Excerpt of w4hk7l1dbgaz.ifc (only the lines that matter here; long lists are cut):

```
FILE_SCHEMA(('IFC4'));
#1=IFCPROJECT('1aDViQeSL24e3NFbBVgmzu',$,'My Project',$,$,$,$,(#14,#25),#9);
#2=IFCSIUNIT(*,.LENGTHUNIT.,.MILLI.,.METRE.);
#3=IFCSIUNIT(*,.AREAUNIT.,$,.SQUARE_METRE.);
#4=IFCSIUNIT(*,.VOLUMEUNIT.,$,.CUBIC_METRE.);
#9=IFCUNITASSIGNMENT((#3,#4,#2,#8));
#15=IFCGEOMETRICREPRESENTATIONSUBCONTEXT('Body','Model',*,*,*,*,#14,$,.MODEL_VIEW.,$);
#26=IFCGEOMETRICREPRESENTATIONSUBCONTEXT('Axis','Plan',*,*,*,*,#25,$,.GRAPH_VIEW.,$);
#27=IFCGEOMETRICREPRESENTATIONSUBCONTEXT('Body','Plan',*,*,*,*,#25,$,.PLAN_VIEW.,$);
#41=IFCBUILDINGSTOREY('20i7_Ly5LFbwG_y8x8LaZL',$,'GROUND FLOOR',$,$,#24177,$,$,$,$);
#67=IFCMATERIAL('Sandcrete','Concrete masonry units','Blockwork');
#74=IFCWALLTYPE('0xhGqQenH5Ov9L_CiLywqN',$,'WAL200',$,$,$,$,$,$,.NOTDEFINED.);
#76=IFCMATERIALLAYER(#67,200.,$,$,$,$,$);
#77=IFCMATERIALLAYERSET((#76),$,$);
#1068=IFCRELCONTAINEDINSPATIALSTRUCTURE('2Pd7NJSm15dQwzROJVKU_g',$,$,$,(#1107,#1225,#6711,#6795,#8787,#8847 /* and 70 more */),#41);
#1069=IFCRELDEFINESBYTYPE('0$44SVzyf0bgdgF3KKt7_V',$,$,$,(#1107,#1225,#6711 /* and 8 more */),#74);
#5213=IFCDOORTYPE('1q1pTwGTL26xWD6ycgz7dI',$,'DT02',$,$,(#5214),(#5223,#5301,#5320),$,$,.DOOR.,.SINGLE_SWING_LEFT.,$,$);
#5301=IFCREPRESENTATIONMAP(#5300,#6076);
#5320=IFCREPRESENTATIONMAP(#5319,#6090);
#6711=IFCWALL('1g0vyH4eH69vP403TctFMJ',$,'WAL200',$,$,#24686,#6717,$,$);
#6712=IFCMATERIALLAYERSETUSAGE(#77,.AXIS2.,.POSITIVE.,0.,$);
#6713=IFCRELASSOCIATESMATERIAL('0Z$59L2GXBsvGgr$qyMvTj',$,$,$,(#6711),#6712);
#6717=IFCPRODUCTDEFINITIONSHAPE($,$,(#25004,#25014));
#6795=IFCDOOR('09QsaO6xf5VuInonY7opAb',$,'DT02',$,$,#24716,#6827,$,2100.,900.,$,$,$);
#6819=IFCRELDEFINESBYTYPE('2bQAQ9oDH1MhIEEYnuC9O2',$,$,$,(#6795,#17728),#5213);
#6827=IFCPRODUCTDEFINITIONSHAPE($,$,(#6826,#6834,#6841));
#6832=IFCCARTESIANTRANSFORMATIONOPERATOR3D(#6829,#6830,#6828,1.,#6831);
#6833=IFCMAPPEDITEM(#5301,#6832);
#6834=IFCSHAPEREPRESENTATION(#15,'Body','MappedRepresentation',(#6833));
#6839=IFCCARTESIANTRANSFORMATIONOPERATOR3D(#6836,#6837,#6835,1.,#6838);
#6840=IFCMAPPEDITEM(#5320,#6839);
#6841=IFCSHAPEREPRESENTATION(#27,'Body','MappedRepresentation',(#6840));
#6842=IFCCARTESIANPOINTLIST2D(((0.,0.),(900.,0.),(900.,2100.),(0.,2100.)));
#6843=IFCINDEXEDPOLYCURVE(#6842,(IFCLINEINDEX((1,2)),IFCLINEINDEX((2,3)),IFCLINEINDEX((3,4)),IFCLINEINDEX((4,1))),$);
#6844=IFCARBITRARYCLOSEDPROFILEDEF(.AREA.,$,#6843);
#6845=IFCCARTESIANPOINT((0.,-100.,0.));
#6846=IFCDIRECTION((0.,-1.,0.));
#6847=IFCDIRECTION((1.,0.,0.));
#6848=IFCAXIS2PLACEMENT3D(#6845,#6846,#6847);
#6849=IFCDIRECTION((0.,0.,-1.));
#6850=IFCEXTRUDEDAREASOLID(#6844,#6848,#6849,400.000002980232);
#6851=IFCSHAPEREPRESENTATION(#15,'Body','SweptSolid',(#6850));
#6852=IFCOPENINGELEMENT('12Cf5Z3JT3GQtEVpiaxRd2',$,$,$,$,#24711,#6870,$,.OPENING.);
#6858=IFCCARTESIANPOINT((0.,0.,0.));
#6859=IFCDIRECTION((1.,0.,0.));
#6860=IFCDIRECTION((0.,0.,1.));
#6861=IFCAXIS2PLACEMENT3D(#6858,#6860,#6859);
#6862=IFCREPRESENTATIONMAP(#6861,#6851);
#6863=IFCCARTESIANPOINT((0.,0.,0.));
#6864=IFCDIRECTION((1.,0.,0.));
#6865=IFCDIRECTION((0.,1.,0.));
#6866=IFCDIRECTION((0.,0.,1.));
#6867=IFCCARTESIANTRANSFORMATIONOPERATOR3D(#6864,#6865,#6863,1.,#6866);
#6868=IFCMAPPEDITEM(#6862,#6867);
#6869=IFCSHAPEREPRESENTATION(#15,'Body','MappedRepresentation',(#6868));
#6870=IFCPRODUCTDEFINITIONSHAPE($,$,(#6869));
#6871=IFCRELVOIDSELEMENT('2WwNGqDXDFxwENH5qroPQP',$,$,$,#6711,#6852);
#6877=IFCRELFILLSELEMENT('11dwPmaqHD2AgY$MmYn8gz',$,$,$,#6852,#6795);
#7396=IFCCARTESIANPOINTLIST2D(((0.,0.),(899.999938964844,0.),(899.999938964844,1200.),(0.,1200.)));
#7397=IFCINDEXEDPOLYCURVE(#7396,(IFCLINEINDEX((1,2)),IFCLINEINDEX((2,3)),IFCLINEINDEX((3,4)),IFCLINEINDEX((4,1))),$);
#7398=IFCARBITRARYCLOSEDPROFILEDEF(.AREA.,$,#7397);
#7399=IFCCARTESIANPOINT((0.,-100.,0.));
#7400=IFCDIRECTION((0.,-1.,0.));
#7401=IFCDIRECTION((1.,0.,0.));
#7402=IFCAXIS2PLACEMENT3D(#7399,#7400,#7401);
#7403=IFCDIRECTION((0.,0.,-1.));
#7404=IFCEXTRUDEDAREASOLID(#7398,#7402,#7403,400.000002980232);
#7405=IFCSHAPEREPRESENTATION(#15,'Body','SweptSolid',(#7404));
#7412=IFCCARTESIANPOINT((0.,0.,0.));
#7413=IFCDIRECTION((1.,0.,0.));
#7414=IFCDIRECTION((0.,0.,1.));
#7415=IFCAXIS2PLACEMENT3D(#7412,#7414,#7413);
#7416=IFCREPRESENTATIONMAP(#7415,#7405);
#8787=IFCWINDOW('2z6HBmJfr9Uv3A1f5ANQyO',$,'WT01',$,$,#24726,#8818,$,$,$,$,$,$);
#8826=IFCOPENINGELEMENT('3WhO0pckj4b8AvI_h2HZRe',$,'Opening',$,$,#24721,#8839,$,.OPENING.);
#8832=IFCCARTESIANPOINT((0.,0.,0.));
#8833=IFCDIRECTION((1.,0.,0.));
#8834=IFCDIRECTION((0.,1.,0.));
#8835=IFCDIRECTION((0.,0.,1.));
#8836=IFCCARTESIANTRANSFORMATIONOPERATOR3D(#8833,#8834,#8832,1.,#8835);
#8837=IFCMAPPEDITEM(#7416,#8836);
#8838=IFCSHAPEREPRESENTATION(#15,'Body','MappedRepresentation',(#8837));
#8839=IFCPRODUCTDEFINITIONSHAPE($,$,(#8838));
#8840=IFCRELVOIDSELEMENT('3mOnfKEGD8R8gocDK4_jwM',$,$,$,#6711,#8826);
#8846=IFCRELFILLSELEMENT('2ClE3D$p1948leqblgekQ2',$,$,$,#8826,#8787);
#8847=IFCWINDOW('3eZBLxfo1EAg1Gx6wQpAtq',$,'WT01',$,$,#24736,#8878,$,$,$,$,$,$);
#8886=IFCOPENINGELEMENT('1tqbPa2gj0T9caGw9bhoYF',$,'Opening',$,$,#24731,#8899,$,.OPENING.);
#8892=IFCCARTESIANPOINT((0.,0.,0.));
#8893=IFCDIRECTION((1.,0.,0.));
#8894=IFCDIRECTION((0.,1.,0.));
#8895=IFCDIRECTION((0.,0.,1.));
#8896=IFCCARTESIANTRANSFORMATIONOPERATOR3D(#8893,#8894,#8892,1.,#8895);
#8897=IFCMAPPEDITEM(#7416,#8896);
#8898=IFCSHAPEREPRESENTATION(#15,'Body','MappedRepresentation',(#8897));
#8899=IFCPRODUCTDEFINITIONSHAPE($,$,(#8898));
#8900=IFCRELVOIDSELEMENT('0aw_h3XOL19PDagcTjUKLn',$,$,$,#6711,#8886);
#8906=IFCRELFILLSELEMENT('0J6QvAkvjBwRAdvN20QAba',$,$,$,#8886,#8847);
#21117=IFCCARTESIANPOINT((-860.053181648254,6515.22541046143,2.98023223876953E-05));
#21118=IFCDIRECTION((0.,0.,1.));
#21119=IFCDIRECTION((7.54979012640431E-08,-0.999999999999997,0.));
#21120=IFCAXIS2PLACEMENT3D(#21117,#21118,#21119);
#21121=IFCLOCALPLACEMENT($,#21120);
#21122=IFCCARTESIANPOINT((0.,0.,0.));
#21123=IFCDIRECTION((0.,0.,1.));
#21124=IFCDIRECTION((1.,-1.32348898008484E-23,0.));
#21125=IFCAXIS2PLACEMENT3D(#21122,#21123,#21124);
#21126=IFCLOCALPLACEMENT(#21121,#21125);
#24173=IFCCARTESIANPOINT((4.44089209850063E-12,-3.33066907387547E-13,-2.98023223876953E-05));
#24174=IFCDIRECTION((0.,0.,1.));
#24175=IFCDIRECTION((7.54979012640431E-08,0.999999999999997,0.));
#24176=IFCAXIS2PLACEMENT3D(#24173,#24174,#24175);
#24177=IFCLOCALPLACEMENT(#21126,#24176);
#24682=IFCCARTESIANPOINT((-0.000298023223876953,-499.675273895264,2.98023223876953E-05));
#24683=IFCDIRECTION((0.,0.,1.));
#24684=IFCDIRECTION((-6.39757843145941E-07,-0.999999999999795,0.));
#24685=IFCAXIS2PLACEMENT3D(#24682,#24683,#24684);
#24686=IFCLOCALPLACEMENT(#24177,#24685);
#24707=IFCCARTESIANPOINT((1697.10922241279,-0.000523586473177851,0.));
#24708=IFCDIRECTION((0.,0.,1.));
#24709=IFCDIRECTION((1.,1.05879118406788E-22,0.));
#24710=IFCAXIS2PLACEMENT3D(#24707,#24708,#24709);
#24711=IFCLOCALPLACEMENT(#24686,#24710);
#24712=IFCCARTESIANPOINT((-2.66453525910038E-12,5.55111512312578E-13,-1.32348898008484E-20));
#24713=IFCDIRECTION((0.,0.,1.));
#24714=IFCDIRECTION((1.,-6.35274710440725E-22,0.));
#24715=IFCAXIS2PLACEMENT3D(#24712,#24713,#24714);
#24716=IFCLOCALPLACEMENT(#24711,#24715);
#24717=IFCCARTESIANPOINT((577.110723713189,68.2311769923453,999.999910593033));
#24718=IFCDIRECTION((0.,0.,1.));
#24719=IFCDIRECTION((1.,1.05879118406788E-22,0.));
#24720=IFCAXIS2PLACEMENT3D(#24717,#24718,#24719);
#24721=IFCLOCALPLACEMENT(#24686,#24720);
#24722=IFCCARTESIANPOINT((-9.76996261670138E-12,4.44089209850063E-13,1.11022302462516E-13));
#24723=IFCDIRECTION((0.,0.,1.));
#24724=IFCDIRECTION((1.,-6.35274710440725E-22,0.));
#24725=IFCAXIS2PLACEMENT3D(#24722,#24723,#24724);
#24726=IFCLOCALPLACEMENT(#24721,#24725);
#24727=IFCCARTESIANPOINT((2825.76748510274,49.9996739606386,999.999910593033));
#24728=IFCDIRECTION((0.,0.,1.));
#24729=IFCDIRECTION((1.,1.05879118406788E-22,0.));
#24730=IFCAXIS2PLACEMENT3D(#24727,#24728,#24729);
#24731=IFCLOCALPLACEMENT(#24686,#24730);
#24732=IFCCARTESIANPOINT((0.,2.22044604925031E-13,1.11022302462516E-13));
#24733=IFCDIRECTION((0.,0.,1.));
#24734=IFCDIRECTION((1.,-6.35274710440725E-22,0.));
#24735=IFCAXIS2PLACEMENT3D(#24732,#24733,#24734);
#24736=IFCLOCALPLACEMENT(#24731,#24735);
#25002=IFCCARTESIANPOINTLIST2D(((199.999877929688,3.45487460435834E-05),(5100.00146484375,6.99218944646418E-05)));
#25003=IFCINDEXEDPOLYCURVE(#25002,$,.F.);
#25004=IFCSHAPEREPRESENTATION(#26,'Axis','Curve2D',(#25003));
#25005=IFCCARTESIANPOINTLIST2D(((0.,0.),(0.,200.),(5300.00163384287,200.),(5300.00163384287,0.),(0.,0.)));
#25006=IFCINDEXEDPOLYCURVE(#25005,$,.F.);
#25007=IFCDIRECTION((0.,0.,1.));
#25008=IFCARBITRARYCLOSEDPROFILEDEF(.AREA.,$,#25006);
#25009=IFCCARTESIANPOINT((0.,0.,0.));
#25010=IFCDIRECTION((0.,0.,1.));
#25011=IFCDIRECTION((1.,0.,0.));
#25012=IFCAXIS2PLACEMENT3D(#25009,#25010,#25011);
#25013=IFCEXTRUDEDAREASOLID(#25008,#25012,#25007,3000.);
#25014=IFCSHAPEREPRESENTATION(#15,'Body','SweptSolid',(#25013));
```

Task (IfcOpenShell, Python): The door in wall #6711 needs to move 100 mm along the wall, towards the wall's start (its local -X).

```python
import ifcopenshell
import ifcopenshell.api.geometry
import ifcopenshell.util.placement

model = ifcopenshell.open("w4hk7l1dbgaz.ifc")

door = model.by_guid("09QsaO6xf5VuInonY7opAb")
opening = door.FillsVoids[0].RelatingOpeningElement
wall = opening.VoidsElements[0].RelatingBuildingElement

wall_matrix = ifcopenshell.util.placement.get_local_placement(wall.ObjectPlacement)
shift = wall_matrix[:3, 0] * -100.0
before = ifcopenshell.util.placement.get_local_placement(door.ObjectPlacement)[:3, 3].copy()

# The door is placed relative to its opening, so it follows when the opening moves.
matrix = ifcopenshell.util.placement.get_local_placement(opening.ObjectPlacement)
matrix[:3, 3] += shift
ifcopenshell.api.geometry.edit_object_placement(
    model, product=opening, matrix=matrix, is_si=False, should_transform_children=True
)

after = ifcopenshell.util.placement.get_local_placement(door.ObjectPlacement)[:3, 3]
print("door moved by", (after - before).round(3) + 0.0)

model.write("w4hk7l1dbgaz_edited.ifc")
```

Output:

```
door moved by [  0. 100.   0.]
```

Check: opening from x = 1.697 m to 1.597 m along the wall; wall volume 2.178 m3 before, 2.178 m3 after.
